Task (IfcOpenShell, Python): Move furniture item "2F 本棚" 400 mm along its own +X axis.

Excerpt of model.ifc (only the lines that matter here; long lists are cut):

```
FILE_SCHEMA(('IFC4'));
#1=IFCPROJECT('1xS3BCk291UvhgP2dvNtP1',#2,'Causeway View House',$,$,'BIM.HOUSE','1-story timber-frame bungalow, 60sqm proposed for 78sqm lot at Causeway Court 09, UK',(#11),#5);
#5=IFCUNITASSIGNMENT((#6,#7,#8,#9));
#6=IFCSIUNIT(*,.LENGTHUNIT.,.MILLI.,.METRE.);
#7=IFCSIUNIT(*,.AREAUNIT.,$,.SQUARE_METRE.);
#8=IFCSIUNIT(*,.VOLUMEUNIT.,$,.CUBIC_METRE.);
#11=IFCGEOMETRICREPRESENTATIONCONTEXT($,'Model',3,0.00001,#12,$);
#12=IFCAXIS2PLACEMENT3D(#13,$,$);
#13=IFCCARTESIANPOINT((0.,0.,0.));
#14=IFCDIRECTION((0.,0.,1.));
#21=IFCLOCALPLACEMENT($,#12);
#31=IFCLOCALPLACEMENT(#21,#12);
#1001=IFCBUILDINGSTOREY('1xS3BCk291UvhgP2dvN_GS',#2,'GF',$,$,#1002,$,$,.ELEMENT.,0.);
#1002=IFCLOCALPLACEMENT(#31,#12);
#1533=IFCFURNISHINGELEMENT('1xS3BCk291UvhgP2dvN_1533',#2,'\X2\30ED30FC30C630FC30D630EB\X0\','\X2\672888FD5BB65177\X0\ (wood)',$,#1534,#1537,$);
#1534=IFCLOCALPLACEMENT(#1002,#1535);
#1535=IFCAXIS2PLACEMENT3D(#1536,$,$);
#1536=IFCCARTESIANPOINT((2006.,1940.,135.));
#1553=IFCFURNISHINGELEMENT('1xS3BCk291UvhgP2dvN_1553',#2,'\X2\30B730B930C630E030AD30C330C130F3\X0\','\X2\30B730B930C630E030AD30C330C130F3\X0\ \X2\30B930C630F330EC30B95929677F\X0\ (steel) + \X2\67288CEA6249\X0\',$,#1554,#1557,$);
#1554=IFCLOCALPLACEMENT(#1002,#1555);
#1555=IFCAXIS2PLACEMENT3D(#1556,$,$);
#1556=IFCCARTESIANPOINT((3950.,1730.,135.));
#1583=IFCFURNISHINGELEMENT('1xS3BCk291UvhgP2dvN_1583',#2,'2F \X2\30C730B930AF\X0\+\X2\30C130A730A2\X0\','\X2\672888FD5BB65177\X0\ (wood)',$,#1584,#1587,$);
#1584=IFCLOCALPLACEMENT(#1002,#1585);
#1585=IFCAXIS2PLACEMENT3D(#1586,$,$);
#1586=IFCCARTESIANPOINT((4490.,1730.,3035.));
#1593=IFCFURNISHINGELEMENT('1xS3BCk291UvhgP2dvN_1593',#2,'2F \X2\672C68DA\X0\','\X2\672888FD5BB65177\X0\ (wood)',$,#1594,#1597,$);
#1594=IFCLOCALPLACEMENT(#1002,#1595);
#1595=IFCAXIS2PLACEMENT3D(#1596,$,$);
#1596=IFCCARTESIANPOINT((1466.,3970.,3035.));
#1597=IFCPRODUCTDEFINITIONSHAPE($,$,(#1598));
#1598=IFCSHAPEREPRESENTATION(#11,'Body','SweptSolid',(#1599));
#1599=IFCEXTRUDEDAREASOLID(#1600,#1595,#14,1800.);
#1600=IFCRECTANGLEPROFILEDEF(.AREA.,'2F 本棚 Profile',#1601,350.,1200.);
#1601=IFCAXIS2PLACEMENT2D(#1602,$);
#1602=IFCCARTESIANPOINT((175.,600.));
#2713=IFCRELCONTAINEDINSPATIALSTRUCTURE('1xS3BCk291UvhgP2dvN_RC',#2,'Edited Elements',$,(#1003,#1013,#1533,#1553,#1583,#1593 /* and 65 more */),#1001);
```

```python
import ifcopenshell
import ifcopenshell.api.geometry
import ifcopenshell.util.placement
import ifcopenshell.util.unit

model = ifcopenshell.open("model.ifc")
unit_scale = ifcopenshell.util.unit.calculate_unit_scale(model)

item = model.by_guid("1xS3BCk291UvhgP2dvN_1593")
matrix = ifcopenshell.util.placement.get_local_placement(item.ObjectPlacement)
matrix[:3, 3] += matrix[:3, 0] * 0.4 / unit_scale
ifcopenshell.api.geometry.edit_object_placement(model, product=item, matrix=matrix, is_si=False)

print(ifcopenshell.util.placement.get_local_placement(item.ObjectPlacement).round(3) + 0.0)

model.write("model_updated.ifc")
```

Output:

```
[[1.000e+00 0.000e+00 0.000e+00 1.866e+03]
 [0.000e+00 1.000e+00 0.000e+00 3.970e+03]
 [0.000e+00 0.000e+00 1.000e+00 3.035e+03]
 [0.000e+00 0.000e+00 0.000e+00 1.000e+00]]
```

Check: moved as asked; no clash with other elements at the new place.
